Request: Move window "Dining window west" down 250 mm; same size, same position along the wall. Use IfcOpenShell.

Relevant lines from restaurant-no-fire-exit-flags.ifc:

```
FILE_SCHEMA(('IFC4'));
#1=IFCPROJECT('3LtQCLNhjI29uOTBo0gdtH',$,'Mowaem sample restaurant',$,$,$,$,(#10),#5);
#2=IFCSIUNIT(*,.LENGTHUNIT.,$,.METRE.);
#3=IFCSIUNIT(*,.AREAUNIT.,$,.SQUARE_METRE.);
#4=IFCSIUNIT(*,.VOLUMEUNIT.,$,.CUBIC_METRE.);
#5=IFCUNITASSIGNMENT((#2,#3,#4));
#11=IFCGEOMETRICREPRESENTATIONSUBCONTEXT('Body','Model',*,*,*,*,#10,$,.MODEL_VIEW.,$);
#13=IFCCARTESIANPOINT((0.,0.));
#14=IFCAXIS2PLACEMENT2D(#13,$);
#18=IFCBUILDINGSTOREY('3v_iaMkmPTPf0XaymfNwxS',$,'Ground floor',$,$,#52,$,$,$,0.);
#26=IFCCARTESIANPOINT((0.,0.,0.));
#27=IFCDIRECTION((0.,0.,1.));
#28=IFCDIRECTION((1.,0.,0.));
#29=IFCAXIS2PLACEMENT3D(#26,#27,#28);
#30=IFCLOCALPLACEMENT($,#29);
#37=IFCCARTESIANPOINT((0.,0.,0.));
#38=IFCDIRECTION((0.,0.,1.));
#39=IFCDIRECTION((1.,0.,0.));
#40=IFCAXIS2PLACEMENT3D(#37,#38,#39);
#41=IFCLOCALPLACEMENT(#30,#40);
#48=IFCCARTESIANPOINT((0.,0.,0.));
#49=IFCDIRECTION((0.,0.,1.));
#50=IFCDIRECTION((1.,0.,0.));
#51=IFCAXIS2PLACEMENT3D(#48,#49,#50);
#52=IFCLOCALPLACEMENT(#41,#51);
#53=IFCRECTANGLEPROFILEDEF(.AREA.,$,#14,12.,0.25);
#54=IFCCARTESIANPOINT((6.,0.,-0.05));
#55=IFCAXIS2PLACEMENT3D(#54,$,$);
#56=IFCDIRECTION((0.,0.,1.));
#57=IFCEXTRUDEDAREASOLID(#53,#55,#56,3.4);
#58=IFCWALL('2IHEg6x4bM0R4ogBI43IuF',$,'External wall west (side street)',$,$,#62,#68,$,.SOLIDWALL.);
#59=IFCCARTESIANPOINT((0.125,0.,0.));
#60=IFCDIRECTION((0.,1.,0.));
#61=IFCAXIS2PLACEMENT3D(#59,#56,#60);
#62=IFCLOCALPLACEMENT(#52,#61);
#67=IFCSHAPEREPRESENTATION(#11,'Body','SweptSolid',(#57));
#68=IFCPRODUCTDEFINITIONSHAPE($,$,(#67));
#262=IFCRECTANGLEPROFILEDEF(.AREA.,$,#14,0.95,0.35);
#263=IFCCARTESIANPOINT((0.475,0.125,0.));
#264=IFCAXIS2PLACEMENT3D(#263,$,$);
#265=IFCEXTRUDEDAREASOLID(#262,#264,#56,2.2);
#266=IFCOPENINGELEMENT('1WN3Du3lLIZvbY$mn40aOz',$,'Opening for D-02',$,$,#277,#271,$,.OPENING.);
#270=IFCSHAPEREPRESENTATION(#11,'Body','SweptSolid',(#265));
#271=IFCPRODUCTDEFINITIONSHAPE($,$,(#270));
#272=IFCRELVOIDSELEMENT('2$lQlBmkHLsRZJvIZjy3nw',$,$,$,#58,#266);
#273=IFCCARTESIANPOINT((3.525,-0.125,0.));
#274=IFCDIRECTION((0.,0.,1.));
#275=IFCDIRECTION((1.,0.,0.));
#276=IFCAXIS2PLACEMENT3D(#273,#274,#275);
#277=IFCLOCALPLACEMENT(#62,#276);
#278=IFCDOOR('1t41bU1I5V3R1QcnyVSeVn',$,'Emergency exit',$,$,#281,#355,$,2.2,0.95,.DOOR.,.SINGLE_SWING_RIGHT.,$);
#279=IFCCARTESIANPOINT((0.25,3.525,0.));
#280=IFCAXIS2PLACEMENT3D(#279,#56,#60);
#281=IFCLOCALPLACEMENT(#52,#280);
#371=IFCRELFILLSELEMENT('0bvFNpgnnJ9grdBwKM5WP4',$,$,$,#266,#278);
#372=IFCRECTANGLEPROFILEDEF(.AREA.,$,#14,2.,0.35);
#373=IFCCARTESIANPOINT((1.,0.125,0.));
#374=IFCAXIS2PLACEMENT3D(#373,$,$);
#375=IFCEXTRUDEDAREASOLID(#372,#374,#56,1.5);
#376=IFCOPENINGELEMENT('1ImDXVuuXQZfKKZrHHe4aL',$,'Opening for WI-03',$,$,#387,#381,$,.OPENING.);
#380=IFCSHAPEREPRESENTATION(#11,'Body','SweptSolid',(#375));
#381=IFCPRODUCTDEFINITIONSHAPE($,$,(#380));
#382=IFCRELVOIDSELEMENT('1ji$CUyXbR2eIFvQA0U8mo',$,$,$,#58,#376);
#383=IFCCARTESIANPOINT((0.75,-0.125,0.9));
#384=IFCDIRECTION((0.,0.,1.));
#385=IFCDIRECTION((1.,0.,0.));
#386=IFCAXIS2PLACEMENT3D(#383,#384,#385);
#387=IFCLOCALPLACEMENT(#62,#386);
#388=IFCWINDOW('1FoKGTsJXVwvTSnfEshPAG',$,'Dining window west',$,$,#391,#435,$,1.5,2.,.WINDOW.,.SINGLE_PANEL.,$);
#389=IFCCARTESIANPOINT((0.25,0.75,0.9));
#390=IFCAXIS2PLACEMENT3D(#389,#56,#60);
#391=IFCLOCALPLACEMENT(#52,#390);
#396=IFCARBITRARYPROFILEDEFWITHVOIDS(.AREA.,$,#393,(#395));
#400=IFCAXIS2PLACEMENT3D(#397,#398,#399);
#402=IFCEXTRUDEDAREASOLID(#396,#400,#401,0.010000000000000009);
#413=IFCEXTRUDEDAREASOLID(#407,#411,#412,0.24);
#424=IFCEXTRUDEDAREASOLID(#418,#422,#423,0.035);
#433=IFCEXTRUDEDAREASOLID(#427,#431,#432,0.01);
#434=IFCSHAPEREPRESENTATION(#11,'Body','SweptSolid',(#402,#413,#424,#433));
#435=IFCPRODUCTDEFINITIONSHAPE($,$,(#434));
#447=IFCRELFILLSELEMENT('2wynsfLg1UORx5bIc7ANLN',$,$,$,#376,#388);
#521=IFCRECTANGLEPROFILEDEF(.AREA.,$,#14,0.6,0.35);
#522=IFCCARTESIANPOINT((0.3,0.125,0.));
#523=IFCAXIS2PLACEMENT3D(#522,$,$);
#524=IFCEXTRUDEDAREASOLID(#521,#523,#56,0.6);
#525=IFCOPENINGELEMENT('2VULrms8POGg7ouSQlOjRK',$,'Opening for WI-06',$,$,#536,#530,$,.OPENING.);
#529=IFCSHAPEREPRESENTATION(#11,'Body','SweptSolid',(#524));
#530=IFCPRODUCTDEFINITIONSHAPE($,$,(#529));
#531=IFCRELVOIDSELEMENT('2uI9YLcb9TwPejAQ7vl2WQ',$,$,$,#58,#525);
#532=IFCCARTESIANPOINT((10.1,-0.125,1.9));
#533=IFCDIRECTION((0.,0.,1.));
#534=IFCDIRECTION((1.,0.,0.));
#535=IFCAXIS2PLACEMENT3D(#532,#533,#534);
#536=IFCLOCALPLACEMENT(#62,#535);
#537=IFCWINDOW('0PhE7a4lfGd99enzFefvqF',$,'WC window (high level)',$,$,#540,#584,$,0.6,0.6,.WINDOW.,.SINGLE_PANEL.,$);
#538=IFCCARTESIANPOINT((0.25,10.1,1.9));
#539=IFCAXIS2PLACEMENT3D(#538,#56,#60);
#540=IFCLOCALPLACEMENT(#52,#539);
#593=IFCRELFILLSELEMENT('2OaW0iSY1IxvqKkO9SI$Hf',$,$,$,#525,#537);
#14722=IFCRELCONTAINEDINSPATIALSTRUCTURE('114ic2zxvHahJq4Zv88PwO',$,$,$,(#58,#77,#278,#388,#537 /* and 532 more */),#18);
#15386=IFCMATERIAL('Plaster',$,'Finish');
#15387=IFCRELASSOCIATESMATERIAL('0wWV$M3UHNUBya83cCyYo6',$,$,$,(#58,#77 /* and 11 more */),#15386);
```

```python
import numpy as np
import ifcopenshell
import ifcopenshell.api.geometry
import ifcopenshell.util.placement
import ifcopenshell.util.unit

model = ifcopenshell.open("restaurant-no-fire-exit-flags.ifc")
unit_scale = ifcopenshell.util.unit.calculate_unit_scale(model)

window = model.by_id(388)
opening = window.FillsVoids[0].RelatingOpeningElement
dz = -0.25

shift = np.array([0.0, 0.0, dz])
# The window is not placed relative to its opening, so move both.
for product in (opening, window):
    matrix = ifcopenshell.util.placement.get_local_placement(product.ObjectPlacement)
    matrix[:3, 3] += shift
    ifcopenshell.api.geometry.edit_object_placement(model, product=product, matrix=matrix, is_si=False)

print(f"moved by {dz * unit_scale:+.3f} m")

model.write("restaurant-no-fire-exit-flags_edited.ifc")
```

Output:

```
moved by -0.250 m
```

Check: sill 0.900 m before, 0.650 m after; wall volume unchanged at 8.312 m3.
